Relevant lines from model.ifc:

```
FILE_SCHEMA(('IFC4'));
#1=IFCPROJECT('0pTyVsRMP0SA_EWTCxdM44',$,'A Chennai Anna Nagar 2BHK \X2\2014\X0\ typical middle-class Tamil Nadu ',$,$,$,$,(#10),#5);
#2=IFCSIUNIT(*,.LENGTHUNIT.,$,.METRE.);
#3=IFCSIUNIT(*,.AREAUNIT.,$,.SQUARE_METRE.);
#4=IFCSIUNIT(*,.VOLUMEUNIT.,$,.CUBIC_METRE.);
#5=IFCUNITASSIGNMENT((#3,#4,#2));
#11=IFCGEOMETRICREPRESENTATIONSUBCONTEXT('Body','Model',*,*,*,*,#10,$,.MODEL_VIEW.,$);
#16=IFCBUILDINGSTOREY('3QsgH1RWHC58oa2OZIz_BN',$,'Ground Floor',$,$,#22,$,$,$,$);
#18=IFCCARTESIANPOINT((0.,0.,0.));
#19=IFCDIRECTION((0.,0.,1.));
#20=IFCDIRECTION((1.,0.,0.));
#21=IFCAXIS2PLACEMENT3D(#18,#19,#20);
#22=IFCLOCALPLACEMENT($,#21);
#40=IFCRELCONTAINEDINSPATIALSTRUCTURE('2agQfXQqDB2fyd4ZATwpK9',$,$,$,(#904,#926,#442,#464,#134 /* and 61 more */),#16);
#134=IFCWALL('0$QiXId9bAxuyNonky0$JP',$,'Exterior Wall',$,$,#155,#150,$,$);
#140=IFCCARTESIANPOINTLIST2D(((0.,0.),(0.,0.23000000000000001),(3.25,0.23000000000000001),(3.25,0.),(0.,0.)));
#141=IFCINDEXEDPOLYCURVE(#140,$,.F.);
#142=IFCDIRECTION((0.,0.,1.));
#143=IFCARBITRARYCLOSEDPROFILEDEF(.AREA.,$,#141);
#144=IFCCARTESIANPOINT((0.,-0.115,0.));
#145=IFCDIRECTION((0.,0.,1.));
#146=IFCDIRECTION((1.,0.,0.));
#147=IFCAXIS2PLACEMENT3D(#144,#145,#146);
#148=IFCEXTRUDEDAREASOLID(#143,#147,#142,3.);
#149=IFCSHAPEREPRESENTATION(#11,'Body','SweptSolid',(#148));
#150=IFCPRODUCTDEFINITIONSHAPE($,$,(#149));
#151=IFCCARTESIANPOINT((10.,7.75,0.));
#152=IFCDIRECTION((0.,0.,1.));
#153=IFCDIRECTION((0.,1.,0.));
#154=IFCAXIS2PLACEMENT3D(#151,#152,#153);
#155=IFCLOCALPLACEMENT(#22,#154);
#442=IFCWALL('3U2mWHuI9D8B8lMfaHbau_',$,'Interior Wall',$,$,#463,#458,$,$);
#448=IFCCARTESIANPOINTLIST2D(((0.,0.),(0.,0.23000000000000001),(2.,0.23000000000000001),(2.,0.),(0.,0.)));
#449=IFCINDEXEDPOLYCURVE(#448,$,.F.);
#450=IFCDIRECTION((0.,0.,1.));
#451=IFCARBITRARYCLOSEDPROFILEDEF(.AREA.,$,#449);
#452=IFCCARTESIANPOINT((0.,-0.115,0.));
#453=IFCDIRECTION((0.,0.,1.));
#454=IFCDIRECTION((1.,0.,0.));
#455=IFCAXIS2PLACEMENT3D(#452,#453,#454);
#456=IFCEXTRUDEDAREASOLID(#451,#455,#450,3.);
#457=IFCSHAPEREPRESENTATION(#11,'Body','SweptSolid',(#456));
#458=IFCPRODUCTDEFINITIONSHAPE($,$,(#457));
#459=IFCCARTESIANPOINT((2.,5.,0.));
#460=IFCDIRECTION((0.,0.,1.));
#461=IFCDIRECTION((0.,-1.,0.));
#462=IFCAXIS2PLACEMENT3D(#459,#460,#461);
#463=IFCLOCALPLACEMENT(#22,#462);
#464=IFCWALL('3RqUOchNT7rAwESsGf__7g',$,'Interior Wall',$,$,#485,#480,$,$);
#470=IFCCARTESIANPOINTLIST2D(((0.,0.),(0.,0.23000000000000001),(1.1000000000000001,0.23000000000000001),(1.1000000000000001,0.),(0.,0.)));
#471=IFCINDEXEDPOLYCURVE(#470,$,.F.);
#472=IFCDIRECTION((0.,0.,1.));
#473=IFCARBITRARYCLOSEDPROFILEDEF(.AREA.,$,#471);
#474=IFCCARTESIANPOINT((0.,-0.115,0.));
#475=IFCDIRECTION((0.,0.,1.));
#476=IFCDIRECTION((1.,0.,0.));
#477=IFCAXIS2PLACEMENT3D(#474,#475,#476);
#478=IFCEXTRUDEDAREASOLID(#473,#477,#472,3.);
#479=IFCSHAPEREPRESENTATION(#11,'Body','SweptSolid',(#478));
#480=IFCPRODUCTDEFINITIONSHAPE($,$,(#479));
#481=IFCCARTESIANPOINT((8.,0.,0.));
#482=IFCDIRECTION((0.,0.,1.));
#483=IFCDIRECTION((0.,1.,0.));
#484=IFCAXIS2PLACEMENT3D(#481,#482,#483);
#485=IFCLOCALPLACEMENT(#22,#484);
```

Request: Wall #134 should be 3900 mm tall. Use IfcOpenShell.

```python
import ifcopenshell
import ifcopenshell.geom
import ifcopenshell.util.representation
import ifcopenshell.util.shape
import ifcopenshell.util.unit

model = ifcopenshell.open("model.ifc")
unit_scale = ifcopenshell.util.unit.calculate_unit_scale(model)
settings = ifcopenshell.geom.settings()


def volume(element):
    """Net volume in cubic metres, openings subtracted."""
    shape = ifcopenshell.geom.create_shape(settings, element)
    return ifcopenshell.util.shape.get_volume(shape.geometry)


wall = model.by_id(134)
before = volume(wall)

body = ifcopenshell.util.representation.get_representation(wall, "Model", "Body")
solid = body.Items[0]
old_height = solid.Depth
solid.Depth = 3.9 / unit_scale
after = volume(wall)

print(f"height {old_height:g} -> {solid.Depth:g}, volume {before:.3f} -> {after:.3f} m3")

model.write("model_edited.ifc")
```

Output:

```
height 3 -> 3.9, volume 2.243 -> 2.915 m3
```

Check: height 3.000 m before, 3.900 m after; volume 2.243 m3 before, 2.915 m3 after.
